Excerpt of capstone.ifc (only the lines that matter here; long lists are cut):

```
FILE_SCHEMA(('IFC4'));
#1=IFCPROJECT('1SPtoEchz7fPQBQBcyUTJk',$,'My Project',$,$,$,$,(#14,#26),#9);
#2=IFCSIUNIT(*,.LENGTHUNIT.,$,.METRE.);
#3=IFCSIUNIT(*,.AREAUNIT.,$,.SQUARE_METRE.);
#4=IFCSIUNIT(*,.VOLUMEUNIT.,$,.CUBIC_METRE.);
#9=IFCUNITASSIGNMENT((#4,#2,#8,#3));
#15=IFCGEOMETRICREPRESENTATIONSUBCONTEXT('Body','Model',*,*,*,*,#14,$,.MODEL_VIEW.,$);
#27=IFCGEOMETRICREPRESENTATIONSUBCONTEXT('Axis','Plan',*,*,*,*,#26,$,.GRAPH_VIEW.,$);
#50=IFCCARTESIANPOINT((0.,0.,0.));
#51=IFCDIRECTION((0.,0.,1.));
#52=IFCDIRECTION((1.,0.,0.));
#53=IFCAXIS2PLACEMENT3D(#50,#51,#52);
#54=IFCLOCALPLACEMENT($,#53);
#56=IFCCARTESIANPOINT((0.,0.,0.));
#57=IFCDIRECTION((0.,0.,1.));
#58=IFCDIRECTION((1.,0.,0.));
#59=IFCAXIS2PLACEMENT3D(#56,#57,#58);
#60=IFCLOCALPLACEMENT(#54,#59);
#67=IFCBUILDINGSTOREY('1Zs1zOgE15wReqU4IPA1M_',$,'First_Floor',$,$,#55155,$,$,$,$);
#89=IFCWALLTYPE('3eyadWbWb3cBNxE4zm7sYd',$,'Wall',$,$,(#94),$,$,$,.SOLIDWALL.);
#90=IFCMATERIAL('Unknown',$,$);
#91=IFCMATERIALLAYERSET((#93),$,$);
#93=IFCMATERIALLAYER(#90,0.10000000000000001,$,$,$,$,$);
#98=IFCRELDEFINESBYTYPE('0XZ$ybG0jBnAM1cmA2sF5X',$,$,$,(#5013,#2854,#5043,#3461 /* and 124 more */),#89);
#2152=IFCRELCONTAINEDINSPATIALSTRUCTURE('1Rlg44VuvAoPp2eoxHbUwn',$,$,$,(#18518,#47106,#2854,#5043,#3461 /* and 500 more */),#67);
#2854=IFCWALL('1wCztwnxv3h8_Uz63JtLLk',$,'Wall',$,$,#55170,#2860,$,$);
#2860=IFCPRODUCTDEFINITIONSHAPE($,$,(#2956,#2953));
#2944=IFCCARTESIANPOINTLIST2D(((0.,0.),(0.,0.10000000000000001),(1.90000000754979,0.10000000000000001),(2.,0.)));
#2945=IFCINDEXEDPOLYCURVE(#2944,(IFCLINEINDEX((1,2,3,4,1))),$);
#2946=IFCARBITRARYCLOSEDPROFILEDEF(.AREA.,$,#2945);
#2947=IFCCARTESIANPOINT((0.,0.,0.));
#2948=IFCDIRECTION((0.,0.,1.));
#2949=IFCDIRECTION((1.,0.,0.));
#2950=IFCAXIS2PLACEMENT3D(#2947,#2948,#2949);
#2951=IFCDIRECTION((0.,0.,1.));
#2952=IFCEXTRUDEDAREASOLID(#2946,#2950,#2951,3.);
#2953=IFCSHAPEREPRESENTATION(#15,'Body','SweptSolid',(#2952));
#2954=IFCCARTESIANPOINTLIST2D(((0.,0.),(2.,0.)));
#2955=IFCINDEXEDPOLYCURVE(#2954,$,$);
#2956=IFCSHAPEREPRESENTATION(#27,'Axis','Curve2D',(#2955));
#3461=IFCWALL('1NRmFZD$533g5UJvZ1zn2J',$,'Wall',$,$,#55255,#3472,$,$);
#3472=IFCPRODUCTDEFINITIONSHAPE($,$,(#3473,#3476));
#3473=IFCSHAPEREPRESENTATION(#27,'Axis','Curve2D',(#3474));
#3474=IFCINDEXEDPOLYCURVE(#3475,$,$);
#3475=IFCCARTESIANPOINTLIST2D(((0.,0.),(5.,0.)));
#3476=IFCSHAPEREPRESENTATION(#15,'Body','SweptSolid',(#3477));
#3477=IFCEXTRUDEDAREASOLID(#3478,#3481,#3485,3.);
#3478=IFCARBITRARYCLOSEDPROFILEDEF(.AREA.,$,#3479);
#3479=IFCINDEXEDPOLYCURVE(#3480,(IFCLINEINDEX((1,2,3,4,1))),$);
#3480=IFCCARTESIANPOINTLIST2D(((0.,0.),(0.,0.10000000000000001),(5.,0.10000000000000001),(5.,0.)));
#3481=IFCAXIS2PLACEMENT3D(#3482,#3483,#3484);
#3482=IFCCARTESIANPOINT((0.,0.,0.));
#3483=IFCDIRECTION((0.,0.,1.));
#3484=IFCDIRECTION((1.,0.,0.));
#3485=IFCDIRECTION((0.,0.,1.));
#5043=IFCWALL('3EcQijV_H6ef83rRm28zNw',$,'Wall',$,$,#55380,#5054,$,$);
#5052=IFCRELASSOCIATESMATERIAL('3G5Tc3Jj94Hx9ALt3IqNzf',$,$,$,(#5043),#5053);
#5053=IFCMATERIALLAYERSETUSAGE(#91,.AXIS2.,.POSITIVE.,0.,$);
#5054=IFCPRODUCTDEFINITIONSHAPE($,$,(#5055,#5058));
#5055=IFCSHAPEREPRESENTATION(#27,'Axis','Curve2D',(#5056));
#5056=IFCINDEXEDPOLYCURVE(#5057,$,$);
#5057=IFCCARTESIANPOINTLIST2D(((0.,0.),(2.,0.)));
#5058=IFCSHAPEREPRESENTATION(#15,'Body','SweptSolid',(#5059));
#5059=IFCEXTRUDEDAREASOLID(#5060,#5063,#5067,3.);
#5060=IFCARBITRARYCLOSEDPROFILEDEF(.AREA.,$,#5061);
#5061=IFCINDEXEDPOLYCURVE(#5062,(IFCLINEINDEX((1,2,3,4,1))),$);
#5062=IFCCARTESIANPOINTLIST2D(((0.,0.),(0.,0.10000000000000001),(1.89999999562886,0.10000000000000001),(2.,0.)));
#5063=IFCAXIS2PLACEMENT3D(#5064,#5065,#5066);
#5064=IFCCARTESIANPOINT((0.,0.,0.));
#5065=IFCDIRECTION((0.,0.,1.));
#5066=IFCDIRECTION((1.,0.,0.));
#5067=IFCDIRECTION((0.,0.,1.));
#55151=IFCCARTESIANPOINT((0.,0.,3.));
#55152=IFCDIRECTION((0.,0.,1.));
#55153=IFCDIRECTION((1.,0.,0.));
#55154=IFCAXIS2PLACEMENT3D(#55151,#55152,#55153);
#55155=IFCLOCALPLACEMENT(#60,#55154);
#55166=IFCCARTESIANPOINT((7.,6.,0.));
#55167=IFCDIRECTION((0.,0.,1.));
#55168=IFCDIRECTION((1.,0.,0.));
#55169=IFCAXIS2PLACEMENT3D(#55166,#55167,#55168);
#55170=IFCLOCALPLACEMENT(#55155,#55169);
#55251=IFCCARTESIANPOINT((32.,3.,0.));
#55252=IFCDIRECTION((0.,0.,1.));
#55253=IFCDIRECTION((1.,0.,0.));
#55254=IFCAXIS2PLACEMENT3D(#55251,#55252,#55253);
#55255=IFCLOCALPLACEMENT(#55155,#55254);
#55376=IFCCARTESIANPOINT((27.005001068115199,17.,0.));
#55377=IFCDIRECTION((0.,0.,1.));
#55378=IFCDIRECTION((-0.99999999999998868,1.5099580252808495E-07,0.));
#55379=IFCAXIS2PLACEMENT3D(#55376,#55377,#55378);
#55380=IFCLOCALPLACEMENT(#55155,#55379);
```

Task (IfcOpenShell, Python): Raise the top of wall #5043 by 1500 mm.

```python
import ifcopenshell
import ifcopenshell.geom
import ifcopenshell.util.representation
import ifcopenshell.util.shape
import ifcopenshell.util.unit

model = ifcopenshell.open("capstone.ifc")
unit_scale = ifcopenshell.util.unit.calculate_unit_scale(model)
settings = ifcopenshell.geom.settings()


def volume(element):
    """Net volume in cubic metres, openings subtracted."""
    shape = ifcopenshell.geom.create_shape(settings, element)
    return ifcopenshell.util.shape.get_volume(shape.geometry)


wall = model.by_id(5043)
before = volume(wall)

body = ifcopenshell.util.representation.get_representation(wall, "Model", "Body")
solid = body.Items[0]
old_height = solid.Depth
solid.Depth += 1.5 / unit_scale
after = volume(wall)

print(f"height {old_height:g} -> {solid.Depth:g}, volume {before:.3f} -> {after:.3f} m3")

model.write("capstone-out.ifc")
```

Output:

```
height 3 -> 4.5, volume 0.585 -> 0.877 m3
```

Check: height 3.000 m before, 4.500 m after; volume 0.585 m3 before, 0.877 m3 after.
